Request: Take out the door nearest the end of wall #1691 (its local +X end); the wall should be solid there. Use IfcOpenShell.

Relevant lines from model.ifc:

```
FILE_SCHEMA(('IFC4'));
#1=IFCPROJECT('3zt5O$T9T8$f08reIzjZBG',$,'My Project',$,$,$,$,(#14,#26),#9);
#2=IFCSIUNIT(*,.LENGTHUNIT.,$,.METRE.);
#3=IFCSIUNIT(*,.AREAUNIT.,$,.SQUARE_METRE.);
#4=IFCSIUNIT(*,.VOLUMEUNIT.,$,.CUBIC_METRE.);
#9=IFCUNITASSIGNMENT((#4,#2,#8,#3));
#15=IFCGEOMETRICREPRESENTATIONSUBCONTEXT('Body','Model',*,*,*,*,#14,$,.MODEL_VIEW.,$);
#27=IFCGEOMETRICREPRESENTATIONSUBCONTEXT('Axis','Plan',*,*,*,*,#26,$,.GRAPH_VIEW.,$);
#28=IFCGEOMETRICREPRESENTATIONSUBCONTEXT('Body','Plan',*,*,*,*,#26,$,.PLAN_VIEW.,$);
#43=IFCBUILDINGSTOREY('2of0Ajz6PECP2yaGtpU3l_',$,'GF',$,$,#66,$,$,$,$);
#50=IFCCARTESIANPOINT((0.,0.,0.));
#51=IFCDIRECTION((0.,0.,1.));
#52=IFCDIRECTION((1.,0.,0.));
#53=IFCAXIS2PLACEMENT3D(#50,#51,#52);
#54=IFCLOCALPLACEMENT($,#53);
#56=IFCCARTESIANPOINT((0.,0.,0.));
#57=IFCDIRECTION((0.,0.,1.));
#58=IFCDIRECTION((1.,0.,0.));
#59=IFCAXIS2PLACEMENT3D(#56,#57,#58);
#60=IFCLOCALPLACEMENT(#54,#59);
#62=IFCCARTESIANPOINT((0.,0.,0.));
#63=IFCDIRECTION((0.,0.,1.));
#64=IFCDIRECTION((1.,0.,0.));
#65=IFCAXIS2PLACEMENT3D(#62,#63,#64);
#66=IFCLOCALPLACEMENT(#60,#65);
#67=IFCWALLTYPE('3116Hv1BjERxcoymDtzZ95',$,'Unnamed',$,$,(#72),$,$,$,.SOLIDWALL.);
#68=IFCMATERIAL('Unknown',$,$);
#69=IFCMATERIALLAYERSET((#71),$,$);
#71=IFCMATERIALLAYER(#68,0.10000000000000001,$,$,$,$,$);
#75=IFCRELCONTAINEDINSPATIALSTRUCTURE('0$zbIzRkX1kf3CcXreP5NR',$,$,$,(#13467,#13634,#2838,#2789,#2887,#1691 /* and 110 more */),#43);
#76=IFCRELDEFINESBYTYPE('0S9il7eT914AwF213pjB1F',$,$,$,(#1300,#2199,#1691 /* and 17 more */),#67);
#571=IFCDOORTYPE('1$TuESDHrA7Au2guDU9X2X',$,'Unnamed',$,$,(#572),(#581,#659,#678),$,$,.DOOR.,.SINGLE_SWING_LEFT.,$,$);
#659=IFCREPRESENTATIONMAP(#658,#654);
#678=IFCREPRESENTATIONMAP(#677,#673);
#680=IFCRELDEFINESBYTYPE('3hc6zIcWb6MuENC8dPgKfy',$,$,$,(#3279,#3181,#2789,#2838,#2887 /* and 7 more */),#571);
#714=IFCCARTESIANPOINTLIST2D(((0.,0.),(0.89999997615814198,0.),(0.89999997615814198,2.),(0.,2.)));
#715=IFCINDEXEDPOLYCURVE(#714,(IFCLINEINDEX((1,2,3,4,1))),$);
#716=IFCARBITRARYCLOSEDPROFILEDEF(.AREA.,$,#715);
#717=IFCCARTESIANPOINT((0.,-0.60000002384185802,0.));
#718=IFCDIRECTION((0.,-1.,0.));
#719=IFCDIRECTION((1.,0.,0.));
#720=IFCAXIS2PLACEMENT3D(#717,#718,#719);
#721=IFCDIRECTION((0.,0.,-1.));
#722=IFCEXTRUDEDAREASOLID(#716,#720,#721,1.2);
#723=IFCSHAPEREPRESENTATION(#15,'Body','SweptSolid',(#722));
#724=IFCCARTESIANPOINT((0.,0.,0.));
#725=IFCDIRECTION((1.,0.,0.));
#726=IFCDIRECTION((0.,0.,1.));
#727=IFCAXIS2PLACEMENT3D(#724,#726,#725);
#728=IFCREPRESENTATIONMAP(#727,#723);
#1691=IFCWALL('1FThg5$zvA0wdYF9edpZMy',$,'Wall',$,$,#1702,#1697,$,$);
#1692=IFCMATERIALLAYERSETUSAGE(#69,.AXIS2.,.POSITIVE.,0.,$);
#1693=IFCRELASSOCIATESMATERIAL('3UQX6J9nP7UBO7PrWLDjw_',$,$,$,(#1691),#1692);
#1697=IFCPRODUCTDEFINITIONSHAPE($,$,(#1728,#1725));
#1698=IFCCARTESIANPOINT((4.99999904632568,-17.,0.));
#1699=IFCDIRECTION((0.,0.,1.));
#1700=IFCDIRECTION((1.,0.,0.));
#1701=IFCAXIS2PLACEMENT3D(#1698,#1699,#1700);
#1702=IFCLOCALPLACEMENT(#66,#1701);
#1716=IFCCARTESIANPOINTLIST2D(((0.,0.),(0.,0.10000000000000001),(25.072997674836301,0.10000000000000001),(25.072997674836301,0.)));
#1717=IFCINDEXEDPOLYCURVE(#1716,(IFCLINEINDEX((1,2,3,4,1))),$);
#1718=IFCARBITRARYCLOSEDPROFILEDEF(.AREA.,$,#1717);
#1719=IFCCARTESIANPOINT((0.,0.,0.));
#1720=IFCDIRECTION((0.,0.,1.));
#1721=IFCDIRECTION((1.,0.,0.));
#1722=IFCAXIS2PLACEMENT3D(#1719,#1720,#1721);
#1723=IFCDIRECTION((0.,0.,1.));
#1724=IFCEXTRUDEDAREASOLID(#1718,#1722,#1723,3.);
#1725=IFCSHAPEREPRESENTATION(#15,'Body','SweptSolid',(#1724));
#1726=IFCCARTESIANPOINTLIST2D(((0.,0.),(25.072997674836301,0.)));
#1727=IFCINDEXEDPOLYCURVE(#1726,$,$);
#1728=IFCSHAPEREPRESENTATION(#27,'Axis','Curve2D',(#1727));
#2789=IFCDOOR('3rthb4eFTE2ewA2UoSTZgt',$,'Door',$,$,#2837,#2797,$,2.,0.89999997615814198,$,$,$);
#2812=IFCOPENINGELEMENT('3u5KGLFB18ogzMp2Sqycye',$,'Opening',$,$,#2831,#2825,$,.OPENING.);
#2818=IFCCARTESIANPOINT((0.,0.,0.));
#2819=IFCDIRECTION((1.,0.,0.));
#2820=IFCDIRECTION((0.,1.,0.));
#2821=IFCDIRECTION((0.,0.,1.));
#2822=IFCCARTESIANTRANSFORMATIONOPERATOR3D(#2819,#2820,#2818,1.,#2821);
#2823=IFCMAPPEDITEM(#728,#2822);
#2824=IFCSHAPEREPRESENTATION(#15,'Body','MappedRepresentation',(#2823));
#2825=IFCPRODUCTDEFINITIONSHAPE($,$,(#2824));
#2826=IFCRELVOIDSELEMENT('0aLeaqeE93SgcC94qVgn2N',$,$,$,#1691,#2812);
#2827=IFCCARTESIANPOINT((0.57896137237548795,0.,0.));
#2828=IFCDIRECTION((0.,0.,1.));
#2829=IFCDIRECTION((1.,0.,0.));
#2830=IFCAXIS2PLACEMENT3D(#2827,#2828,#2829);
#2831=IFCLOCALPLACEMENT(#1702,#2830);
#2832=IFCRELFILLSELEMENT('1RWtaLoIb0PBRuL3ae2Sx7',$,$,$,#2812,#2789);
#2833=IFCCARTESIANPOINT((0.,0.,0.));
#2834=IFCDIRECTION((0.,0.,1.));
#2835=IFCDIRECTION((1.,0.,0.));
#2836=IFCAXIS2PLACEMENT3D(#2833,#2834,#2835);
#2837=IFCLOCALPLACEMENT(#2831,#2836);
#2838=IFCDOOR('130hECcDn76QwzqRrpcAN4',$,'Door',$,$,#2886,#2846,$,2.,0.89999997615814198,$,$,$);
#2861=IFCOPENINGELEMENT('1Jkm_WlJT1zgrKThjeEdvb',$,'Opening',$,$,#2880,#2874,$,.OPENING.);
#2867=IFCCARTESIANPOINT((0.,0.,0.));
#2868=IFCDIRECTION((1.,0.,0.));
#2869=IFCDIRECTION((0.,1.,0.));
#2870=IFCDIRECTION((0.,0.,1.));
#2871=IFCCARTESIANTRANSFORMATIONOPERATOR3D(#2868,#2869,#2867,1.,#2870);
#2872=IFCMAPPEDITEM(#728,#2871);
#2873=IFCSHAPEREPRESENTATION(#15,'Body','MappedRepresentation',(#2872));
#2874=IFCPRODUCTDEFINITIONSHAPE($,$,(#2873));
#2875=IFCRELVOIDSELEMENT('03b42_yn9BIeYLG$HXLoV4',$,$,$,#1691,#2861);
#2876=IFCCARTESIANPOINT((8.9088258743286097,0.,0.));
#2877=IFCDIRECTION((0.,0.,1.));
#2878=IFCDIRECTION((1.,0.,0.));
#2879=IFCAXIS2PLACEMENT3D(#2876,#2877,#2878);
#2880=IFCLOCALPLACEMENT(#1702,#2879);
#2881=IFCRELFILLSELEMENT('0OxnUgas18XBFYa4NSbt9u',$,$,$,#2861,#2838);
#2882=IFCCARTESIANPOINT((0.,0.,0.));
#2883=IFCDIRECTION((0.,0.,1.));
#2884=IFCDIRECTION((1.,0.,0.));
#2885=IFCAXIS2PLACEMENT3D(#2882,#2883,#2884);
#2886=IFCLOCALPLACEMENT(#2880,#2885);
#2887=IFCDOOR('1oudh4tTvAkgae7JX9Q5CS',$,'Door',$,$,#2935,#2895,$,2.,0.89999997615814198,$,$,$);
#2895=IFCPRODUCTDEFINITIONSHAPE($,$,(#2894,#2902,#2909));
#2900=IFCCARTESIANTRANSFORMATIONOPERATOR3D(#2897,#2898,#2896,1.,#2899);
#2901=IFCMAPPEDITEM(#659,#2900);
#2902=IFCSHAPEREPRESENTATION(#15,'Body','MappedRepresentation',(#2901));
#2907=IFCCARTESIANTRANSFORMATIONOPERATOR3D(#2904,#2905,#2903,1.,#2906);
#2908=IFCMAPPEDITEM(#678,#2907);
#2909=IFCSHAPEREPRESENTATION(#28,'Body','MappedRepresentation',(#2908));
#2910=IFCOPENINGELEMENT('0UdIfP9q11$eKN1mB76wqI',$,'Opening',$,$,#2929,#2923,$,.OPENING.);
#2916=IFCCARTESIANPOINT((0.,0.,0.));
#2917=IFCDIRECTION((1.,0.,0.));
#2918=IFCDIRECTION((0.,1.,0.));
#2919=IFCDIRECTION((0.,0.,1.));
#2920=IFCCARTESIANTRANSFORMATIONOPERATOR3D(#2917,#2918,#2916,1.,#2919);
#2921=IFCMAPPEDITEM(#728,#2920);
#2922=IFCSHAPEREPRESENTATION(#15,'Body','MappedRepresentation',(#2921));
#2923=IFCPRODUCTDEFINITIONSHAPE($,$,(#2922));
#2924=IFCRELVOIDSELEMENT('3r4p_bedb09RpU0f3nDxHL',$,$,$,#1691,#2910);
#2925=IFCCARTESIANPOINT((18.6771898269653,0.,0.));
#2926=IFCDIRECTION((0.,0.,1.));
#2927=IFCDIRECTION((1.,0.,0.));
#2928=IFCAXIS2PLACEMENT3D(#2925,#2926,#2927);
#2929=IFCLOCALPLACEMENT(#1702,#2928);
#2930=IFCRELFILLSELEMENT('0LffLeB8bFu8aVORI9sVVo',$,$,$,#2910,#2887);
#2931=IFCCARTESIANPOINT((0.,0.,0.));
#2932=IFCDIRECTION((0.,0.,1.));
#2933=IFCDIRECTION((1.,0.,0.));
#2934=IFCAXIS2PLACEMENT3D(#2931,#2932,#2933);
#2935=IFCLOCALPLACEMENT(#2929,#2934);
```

```python
import ifcopenshell
import ifcopenshell.api.feature
import ifcopenshell.api.root
import ifcopenshell.geom
import ifcopenshell.util.shape

model = ifcopenshell.open("model.ifc")
settings = ifcopenshell.geom.settings()


def volume(element):
    """Net volume in cubic metres, openings subtracted."""
    shape = ifcopenshell.geom.create_shape(settings, element)
    return ifcopenshell.util.shape.get_volume(shape.geometry)


door = model.by_guid("1oudh4tTvAkgae7JX9Q5CS")
opening = door.FillsVoids[0].RelatingOpeningElement
wall = opening.VoidsElements[0].RelatingBuildingElement
before = volume(wall)

ifcopenshell.api.root.remove_product(model, product=door)
ifcopenshell.api.feature.remove_feature(model, feature=opening)

after = volume(wall)

print(f"wall volume {before:.3f} -> {after:.3f} m3")

model.write("model_rev.ifc")
```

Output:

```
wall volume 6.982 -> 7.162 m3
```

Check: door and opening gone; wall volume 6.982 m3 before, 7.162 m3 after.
